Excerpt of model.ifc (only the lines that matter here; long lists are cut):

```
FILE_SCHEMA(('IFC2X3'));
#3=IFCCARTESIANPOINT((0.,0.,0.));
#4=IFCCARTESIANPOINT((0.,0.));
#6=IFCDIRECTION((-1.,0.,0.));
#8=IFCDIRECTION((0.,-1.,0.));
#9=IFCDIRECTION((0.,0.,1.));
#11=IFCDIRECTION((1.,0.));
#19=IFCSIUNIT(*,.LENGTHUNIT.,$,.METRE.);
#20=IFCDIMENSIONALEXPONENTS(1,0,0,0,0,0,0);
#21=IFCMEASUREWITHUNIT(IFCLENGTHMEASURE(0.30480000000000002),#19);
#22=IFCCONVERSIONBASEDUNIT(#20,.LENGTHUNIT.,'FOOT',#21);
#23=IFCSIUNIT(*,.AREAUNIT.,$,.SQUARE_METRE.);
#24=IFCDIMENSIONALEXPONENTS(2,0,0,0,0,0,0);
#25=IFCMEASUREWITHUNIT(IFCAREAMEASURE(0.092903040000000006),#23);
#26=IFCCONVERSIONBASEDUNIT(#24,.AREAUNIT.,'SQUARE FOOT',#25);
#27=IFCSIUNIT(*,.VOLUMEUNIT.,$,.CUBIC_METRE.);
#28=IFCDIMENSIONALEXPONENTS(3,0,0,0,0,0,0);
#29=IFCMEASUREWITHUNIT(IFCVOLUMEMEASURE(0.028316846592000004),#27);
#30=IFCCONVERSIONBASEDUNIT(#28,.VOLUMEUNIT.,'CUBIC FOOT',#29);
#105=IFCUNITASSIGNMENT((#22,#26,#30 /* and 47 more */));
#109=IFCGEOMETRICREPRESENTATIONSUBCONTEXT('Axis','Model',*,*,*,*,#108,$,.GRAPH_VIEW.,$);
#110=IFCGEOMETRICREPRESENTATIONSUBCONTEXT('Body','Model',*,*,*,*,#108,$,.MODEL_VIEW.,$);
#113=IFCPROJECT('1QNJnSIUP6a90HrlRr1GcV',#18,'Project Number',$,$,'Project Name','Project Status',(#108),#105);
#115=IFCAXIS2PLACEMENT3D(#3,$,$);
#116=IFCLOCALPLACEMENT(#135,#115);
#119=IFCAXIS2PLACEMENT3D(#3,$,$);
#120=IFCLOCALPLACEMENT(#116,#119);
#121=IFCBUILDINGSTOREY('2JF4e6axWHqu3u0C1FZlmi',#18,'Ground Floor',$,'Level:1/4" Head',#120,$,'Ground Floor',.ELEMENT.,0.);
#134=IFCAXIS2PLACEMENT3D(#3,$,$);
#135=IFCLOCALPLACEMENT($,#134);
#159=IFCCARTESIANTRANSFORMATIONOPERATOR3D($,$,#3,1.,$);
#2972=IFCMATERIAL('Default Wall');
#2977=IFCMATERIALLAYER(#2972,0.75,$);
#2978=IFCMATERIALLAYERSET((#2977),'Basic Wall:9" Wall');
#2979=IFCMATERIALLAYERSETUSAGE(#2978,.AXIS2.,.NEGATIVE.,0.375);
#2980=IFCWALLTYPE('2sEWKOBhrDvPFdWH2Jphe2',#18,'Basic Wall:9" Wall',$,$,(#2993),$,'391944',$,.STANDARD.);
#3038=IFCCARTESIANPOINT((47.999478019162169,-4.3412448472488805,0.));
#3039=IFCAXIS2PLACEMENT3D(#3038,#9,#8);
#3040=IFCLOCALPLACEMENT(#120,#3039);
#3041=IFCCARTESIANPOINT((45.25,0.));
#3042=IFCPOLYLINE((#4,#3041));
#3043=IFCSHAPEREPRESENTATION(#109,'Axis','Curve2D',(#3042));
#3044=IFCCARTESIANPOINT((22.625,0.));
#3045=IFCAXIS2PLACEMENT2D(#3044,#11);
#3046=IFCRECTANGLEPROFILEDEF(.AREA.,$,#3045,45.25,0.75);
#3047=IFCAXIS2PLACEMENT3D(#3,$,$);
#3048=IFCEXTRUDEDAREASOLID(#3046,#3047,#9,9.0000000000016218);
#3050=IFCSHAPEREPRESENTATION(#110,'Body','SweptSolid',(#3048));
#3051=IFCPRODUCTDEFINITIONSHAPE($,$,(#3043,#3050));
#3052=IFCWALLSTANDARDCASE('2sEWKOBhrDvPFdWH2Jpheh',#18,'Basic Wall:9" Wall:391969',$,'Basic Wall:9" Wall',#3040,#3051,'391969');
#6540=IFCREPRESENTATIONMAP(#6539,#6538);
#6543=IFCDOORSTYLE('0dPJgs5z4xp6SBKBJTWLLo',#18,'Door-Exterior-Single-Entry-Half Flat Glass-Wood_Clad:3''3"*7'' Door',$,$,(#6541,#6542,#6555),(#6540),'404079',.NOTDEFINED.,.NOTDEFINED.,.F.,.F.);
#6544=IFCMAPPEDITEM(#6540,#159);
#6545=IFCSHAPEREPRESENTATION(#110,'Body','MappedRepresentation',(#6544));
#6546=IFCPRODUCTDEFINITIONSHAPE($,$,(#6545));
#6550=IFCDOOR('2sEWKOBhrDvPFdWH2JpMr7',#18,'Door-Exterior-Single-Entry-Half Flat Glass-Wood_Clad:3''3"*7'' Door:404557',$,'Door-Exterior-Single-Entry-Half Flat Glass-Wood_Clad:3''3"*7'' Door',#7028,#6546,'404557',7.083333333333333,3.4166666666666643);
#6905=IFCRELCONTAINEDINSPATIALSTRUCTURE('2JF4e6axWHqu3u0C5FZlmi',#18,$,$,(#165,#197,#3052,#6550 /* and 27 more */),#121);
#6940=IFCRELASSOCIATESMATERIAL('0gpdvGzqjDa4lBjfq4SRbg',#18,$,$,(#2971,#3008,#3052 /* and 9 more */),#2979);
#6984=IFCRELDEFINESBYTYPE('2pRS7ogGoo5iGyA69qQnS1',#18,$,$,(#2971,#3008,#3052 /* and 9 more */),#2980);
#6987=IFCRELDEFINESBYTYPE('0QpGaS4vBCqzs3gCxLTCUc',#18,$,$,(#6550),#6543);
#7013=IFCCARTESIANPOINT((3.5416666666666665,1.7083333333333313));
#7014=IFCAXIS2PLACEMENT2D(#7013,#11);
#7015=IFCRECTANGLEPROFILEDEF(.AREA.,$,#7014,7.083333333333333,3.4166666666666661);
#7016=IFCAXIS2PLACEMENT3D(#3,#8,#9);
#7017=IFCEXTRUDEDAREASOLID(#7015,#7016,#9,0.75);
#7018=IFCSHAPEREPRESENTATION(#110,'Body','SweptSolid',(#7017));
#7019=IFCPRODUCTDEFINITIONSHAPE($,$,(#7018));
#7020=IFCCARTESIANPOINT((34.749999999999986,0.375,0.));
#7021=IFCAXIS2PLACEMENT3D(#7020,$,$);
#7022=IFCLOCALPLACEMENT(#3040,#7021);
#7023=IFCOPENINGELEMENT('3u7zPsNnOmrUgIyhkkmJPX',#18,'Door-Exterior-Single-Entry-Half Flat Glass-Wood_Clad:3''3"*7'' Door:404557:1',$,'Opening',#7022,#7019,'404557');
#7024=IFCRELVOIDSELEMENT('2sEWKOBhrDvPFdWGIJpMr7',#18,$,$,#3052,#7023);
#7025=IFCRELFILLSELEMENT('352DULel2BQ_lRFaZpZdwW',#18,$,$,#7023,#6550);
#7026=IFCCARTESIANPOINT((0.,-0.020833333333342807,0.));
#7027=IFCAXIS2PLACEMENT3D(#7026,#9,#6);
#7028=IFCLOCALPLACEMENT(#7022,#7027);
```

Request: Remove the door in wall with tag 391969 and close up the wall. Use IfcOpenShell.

```python
import ifcopenshell
import ifcopenshell.api.feature
import ifcopenshell.api.root
import ifcopenshell.geom
import ifcopenshell.util.shape

model = ifcopenshell.open("model.ifc")
settings = ifcopenshell.geom.settings()


def volume(element):
    """Net volume in cubic metres, openings subtracted."""
    shape = ifcopenshell.geom.create_shape(settings, element)
    return ifcopenshell.util.shape.get_volume(shape.geometry)


door = model.by_guid("2sEWKOBhrDvPFdWH2JpMr7")
opening = door.FillsVoids[0].RelatingOpeningElement
wall = opening.VoidsElements[0].RelatingBuildingElement
before = volume(wall)

ifcopenshell.api.root.remove_product(model, product=door)
ifcopenshell.api.feature.remove_feature(model, feature=opening)

after = volume(wall)

print(f"wall volume {before:.3f} -> {after:.3f} m3")

model.write("model-out.ifc")
```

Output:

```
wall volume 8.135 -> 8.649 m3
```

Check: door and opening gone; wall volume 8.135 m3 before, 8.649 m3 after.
